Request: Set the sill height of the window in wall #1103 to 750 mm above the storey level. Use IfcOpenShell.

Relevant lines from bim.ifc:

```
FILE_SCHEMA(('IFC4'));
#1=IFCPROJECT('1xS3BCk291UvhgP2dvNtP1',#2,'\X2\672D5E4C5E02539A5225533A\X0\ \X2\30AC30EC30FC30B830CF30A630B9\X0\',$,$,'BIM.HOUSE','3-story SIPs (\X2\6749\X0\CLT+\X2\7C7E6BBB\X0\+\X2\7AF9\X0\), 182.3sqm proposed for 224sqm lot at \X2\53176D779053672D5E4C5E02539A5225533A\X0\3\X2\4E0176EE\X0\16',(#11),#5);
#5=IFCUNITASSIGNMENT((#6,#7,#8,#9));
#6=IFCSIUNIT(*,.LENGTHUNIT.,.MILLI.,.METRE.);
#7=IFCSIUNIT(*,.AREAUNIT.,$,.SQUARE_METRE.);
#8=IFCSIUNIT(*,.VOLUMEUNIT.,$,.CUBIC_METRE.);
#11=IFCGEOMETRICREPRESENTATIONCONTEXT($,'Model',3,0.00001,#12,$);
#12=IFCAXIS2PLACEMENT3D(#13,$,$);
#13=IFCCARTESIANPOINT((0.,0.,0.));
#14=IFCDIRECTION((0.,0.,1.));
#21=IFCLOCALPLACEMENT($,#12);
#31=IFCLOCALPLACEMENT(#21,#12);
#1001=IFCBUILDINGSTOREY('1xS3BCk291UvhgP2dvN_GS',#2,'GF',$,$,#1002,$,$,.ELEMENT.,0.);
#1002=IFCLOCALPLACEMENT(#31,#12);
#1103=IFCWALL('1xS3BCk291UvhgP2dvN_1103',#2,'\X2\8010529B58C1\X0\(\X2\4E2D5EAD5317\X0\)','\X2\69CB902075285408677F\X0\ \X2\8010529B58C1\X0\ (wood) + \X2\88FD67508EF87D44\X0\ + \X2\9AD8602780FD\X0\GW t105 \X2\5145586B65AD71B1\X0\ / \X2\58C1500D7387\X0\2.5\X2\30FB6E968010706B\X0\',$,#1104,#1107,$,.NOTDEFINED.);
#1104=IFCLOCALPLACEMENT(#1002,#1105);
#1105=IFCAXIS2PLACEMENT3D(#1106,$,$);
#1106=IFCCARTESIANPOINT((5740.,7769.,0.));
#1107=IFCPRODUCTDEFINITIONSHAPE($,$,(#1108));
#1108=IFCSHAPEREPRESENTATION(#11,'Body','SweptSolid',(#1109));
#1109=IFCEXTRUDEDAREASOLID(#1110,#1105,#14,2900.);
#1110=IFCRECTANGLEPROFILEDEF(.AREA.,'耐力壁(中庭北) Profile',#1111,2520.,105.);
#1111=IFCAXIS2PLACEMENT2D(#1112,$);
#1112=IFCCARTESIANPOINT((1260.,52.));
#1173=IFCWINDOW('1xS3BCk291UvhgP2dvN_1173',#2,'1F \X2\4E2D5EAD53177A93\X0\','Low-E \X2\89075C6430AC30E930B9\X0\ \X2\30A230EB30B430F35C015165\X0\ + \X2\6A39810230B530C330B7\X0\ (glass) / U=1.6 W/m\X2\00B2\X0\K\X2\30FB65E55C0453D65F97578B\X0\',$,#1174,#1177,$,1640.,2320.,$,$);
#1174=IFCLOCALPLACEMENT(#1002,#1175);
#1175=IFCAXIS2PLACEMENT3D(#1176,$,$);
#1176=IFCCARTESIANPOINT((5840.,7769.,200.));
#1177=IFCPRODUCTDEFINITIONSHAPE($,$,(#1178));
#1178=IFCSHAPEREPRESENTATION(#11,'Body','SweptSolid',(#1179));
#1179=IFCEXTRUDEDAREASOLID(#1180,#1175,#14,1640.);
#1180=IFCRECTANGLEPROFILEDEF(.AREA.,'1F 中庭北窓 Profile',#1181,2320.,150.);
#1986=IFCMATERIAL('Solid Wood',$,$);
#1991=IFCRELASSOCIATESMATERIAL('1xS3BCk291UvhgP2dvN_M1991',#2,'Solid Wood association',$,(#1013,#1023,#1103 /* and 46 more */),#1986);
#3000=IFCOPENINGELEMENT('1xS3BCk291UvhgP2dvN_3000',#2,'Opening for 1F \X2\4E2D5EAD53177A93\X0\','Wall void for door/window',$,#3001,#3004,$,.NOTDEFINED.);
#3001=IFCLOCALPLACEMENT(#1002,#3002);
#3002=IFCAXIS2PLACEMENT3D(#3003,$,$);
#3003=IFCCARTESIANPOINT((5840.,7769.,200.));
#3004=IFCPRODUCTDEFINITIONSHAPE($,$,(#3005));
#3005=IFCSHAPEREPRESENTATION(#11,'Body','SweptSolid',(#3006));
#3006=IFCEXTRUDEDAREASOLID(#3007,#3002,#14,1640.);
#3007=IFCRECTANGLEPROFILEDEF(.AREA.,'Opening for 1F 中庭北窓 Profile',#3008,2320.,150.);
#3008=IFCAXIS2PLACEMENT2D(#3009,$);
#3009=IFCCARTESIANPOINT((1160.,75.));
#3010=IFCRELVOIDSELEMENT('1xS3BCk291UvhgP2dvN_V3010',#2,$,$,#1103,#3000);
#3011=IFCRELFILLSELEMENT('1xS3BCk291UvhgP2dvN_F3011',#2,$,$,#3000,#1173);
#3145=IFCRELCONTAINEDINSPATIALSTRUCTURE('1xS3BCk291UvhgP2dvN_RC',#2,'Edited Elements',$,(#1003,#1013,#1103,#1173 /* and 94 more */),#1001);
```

```python
import numpy as np
import ifcopenshell
import ifcopenshell.api.geometry
import ifcopenshell.geom
import ifcopenshell.util.element
import ifcopenshell.util.placement
import ifcopenshell.util.shape
import ifcopenshell.util.unit

model = ifcopenshell.open("bim.ifc")
unit_scale = ifcopenshell.util.unit.calculate_unit_scale(model)

window = model.by_id(1173)
opening = window.FillsVoids[0].RelatingOpeningElement
storey = ifcopenshell.util.element.get_container(window, ifc_class="IfcBuildingStorey")
level = ifcopenshell.util.placement.get_local_placement(storey.ObjectPlacement)[2, 3]

# The opening's origin need not be at the sill, so measure its lowest point.
shape = ifcopenshell.geom.create_shape(ifcopenshell.geom.settings(), opening)
bottom = ifcopenshell.util.shape.get_shape_bottom_elevation(shape, shape.geometry) / unit_scale
dz = level + 0.75 / unit_scale - bottom

shift = np.array([0.0, 0.0, dz])
# The window is not placed relative to its opening, so move both.
for product in (opening, window):
    matrix = ifcopenshell.util.placement.get_local_placement(product.ObjectPlacement)
    matrix[:3, 3] += shift
    ifcopenshell.api.geometry.edit_object_placement(model, product=product, matrix=matrix, is_si=False)

print(f"moved by {dz * unit_scale:+.3f} m")

model.write("bim_rev.ifc")
```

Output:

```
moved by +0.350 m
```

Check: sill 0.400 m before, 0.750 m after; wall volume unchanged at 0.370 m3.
